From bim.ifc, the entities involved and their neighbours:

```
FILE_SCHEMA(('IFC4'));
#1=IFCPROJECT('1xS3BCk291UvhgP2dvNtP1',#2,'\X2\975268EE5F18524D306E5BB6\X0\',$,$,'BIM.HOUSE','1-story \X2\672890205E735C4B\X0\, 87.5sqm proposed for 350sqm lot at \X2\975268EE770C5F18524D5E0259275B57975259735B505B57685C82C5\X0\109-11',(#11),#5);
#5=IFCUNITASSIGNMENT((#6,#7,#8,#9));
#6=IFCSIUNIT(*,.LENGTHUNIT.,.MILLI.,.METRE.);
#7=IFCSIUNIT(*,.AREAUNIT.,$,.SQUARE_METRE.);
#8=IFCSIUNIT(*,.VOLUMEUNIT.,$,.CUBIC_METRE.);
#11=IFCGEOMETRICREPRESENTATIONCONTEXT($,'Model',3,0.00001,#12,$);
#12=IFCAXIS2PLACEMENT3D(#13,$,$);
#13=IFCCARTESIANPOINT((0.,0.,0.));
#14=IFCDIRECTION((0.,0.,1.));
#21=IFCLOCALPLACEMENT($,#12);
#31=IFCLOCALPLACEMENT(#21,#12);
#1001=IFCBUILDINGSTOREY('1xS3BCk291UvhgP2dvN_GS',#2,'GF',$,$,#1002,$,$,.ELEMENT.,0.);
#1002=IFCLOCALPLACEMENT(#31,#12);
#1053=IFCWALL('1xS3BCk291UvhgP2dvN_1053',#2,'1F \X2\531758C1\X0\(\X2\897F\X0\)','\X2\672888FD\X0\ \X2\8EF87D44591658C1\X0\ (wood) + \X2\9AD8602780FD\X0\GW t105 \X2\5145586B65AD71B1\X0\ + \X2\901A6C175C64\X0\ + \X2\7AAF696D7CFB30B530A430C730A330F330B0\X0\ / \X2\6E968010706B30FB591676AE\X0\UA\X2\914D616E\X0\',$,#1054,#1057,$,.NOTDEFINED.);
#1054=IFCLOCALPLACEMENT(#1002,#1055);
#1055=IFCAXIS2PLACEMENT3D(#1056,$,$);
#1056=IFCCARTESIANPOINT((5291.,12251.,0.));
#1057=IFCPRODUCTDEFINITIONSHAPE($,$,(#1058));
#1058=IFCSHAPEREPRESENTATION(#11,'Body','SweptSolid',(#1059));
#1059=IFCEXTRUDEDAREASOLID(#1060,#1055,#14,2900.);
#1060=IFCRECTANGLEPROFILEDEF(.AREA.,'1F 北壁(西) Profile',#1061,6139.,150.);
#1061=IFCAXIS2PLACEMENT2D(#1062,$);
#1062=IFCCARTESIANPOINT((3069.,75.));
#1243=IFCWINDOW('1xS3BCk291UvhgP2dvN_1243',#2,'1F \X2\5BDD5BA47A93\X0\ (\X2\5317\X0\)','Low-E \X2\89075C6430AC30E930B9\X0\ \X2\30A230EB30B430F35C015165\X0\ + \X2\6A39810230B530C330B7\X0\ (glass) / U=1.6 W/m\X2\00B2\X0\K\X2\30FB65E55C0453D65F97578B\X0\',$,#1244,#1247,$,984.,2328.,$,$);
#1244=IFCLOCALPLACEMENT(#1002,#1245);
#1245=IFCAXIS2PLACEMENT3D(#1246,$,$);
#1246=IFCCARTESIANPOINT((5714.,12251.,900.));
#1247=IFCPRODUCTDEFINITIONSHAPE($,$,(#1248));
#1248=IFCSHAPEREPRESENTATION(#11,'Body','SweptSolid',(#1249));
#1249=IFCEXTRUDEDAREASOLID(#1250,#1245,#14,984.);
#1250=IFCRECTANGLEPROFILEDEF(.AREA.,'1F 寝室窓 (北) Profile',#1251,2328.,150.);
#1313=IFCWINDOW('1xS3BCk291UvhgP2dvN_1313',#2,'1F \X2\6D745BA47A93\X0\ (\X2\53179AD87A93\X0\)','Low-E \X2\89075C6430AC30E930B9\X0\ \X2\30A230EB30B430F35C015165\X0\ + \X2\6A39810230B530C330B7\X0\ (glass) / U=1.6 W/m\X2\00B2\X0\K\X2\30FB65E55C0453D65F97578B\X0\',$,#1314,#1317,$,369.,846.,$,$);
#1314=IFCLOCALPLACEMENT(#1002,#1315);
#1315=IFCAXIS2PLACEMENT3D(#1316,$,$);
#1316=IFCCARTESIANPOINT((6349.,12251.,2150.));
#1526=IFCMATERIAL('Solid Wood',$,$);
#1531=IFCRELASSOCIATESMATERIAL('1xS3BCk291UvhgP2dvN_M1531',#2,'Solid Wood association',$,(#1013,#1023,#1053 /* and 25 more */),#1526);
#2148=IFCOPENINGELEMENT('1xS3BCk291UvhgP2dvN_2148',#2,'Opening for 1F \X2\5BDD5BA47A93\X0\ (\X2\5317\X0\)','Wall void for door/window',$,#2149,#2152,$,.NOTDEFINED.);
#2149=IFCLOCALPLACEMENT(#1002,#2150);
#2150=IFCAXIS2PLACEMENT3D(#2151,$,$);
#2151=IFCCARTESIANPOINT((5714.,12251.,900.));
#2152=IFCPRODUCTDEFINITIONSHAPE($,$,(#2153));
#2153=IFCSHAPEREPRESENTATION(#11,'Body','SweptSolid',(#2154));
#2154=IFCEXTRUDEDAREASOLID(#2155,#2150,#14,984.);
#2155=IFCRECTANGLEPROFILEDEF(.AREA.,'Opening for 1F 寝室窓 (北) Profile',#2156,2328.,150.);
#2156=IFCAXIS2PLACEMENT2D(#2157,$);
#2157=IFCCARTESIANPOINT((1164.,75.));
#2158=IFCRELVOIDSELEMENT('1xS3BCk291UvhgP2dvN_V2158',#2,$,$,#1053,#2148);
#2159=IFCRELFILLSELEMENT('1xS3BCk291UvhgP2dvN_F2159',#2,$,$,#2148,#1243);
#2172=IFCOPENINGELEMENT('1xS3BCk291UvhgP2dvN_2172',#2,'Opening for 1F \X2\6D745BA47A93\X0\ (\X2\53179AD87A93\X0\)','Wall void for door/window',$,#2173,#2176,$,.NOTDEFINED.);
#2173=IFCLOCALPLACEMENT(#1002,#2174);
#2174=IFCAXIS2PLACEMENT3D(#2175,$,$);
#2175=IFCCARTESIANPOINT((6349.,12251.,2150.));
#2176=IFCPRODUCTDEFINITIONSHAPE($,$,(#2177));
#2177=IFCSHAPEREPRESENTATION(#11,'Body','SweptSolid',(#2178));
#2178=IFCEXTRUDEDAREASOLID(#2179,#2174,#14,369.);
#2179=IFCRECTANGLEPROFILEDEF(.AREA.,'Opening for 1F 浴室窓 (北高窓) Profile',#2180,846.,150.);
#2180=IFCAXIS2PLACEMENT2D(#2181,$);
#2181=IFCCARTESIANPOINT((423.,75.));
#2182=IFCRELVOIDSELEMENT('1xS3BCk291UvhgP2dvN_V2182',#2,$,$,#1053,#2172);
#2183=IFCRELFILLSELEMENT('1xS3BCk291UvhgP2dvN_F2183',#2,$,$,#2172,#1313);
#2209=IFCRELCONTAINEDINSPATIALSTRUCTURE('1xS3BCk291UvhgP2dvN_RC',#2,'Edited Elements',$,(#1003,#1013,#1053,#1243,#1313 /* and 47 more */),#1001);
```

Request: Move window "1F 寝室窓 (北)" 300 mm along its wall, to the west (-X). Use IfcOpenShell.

```python
import ifcopenshell
import ifcopenshell.api.geometry
import ifcopenshell.util.placement

model = ifcopenshell.open("bim.ifc")

window = model.by_guid("1xS3BCk291UvhgP2dvN_1243")
opening = window.FillsVoids[0].RelatingOpeningElement
wall = opening.VoidsElements[0].RelatingBuildingElement

wall_matrix = ifcopenshell.util.placement.get_local_placement(wall.ObjectPlacement)
shift = wall_matrix[:3, 0] * -300.0
before = ifcopenshell.util.placement.get_local_placement(window.ObjectPlacement)[:3, 3].copy()

# The window is not placed relative to its opening, so move both.
for product in (opening, window):
    matrix = ifcopenshell.util.placement.get_local_placement(product.ObjectPlacement)
    matrix[:3, 3] += shift
    ifcopenshell.api.geometry.edit_object_placement(model, product=product, matrix=matrix, is_si=False)

after = ifcopenshell.util.placement.get_local_placement(window.ObjectPlacement)[:3, 3]
print("window moved by", (after - before).round(3) + 0.0)

model.write("bim_updated.ifc")
```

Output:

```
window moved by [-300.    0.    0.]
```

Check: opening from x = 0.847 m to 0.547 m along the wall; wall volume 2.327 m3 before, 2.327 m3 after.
